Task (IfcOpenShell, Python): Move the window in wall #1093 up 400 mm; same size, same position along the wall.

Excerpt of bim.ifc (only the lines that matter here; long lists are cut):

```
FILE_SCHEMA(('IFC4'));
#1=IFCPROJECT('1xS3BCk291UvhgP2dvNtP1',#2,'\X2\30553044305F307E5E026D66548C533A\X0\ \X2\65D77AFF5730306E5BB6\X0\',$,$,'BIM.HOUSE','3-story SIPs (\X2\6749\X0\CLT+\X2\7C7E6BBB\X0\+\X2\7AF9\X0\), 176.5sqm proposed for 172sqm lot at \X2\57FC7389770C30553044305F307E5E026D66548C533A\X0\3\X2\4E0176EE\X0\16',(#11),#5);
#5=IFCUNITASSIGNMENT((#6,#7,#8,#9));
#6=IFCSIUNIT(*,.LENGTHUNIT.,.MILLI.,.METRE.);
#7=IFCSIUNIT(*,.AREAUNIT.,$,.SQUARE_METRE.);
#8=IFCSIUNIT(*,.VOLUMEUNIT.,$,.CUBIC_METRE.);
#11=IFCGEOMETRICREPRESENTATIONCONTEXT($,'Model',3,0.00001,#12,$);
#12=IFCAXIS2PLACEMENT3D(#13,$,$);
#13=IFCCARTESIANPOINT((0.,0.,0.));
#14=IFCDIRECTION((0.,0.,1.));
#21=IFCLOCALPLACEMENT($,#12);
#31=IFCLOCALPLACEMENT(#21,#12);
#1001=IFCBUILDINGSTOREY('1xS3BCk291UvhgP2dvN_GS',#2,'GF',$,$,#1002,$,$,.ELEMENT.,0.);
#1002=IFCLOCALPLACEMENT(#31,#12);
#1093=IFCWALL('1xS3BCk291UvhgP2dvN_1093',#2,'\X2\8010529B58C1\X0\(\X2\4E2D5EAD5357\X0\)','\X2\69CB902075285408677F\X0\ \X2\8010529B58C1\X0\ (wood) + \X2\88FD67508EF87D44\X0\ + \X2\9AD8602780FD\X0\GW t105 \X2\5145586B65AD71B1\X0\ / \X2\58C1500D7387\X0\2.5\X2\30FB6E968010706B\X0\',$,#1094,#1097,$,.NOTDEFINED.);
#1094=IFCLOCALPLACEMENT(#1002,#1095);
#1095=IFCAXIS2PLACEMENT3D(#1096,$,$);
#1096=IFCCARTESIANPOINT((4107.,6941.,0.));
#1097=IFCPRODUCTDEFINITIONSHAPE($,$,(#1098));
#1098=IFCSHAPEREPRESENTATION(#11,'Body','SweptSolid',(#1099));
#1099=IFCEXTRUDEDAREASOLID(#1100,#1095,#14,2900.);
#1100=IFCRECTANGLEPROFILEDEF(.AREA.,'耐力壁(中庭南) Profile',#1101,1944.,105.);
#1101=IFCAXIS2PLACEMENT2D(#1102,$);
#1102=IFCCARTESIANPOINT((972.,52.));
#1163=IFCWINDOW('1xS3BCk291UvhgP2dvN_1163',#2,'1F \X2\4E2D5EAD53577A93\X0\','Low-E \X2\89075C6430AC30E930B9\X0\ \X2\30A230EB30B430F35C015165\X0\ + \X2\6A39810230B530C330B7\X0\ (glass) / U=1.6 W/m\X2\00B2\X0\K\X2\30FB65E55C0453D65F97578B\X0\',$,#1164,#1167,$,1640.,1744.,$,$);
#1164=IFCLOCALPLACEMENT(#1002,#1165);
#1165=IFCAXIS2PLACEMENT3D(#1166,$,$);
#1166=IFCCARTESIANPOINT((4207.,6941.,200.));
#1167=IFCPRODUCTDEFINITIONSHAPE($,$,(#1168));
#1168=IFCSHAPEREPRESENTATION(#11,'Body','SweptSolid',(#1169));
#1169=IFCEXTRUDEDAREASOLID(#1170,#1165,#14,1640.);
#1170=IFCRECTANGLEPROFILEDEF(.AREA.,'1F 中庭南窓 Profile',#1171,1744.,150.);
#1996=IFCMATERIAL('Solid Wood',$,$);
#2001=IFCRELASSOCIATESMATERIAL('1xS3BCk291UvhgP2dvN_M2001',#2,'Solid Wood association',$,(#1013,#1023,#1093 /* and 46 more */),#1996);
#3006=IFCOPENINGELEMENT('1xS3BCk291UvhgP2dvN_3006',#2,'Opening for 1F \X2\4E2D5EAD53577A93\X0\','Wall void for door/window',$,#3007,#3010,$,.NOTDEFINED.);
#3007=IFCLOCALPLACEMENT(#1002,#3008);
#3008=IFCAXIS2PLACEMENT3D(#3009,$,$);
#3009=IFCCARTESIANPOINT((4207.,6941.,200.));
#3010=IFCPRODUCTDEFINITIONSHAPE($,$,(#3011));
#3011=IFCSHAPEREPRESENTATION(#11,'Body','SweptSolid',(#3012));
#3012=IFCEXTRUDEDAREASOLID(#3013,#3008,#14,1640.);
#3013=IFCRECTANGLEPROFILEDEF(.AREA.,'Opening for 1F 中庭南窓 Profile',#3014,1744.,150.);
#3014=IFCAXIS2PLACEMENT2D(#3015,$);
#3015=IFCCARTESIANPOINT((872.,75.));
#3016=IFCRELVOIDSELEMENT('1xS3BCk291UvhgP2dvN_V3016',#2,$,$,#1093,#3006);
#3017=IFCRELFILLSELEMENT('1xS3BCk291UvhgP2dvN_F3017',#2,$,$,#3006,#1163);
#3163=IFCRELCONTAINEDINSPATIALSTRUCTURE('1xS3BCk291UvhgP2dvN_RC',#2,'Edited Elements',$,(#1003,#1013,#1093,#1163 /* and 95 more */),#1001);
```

```python
import numpy as np
import ifcopenshell
import ifcopenshell.api.geometry
import ifcopenshell.util.placement
import ifcopenshell.util.unit

model = ifcopenshell.open("bim.ifc")
unit_scale = ifcopenshell.util.unit.calculate_unit_scale(model)

window = model.by_guid("1xS3BCk291UvhgP2dvN_1163")
opening = window.FillsVoids[0].RelatingOpeningElement
dz = 400.0

shift = np.array([0.0, 0.0, dz])
# The window is not placed relative to its opening, so move both.
for product in (opening, window):
    matrix = ifcopenshell.util.placement.get_local_placement(product.ObjectPlacement)
    matrix[:3, 3] += shift
    ifcopenshell.api.geometry.edit_object_placement(model, product=product, matrix=matrix, is_si=False)

print(f"moved by {dz * unit_scale:+.3f} m")

model.write("bim-out.ifc")
```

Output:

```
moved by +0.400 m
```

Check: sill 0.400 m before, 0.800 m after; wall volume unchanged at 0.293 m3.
